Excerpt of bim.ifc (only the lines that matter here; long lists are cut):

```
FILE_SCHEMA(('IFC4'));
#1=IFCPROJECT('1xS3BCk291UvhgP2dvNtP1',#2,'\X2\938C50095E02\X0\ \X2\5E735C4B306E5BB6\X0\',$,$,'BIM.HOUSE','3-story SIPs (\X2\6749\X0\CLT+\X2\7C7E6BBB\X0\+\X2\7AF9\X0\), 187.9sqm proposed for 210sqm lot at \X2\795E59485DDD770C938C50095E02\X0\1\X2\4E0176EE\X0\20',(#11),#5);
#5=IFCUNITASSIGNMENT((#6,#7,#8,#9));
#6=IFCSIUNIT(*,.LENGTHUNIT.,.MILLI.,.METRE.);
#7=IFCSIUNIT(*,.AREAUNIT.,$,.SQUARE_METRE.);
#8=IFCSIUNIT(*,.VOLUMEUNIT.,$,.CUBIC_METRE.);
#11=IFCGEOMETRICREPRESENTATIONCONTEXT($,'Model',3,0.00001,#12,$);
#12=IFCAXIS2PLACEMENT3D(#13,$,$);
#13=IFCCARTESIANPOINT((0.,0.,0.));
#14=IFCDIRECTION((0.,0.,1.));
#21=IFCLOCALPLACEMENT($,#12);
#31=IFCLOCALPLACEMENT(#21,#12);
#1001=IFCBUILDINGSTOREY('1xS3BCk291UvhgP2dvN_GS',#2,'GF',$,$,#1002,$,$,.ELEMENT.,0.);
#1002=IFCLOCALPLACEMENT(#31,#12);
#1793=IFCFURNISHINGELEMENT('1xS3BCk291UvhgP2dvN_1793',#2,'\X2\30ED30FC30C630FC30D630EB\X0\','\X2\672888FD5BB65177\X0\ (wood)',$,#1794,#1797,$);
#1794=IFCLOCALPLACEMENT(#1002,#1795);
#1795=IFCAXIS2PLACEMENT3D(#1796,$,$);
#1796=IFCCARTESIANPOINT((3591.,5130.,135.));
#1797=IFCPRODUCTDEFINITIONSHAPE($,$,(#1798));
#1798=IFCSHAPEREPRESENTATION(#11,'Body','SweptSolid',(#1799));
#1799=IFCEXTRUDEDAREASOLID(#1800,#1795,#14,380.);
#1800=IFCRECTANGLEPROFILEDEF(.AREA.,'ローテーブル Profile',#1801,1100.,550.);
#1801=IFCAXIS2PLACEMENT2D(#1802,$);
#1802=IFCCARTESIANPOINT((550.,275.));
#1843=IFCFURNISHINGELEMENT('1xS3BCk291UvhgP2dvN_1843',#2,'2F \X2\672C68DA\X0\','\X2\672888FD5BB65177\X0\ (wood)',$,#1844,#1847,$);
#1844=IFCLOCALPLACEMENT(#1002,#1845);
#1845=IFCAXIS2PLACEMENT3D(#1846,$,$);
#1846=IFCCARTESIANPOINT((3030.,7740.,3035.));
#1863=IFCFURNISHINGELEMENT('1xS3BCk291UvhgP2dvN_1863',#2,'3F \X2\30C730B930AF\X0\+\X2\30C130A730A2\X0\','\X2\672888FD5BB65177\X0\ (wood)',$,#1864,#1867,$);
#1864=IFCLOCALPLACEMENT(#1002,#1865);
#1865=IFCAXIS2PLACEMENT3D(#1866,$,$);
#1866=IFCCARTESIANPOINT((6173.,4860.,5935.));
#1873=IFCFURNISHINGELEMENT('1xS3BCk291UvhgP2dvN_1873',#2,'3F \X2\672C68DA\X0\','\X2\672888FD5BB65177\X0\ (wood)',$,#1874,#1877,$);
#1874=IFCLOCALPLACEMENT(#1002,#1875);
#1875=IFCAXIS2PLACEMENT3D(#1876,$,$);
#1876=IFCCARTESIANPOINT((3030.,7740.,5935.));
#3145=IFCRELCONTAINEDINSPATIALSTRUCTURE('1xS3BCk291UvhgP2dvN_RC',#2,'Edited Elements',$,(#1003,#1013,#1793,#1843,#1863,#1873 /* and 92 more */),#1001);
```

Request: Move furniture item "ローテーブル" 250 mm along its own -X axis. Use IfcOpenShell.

```python
import ifcopenshell
import ifcopenshell.api.geometry
import ifcopenshell.util.placement

model = ifcopenshell.open("bim.ifc")

item = model.by_guid("1xS3BCk291UvhgP2dvN_1793")
matrix = ifcopenshell.util.placement.get_local_placement(item.ObjectPlacement)
matrix[:3, 3] -= matrix[:3, 0] * 250.0
ifcopenshell.api.geometry.edit_object_placement(model, product=item, matrix=matrix, is_si=False)

print(ifcopenshell.util.placement.get_local_placement(item.ObjectPlacement).round(3) + 0.0)

model.write("bim_v2.ifc")
```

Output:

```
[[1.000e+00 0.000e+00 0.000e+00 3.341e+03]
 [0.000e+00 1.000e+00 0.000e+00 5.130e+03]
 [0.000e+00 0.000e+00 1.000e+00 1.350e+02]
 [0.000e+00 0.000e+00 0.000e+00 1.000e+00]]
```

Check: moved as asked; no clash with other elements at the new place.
